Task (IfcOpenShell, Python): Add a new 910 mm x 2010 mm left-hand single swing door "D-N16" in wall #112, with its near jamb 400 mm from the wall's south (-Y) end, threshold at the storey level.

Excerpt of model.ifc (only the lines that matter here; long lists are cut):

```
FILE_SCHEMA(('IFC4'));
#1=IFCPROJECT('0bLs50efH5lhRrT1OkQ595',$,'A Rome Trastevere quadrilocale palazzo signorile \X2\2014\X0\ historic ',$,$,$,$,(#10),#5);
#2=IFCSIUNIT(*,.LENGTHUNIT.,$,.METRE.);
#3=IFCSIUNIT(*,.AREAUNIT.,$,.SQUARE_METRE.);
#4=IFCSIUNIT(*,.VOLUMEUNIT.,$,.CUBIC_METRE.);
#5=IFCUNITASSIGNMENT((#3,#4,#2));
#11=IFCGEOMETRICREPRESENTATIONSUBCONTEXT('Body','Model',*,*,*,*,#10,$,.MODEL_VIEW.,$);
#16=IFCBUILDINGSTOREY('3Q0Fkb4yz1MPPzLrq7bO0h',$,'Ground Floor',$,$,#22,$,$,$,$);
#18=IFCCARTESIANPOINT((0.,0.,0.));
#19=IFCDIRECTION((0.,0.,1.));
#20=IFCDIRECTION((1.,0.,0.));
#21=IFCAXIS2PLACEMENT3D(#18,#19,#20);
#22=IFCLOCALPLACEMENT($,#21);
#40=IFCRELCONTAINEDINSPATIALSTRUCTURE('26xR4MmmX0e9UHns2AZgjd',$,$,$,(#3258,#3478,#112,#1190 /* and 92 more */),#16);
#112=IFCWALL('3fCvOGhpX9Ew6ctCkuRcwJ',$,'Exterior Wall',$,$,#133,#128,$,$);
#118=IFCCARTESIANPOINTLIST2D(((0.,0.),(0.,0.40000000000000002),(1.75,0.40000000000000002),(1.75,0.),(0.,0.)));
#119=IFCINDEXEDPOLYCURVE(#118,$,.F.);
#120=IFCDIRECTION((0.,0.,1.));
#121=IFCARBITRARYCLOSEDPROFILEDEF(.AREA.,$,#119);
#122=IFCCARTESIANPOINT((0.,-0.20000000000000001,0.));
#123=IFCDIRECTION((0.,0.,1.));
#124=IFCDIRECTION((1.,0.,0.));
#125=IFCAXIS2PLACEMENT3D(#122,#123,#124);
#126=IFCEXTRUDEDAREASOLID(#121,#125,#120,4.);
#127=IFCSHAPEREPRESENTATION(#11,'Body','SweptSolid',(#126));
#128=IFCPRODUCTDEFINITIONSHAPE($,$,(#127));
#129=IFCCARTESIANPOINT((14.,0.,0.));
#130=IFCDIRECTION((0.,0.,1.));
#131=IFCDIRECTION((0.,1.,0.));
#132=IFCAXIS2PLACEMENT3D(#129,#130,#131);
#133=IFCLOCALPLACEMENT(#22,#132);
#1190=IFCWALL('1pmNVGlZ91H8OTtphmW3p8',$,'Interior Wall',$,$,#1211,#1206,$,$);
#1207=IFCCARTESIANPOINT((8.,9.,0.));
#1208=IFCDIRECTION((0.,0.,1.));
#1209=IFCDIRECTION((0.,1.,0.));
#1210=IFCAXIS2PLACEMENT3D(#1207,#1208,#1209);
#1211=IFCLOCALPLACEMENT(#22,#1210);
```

```python
import numpy as np
import ifcopenshell
import ifcopenshell.api.feature
import ifcopenshell.api.geometry
import ifcopenshell.api.root
import ifcopenshell.api.spatial
import ifcopenshell.geom
import ifcopenshell.util.element
import ifcopenshell.util.placement
import ifcopenshell.util.representation
import ifcopenshell.util.shape
import ifcopenshell.util.unit

model = ifcopenshell.open("model.ifc")
unit_scale = ifcopenshell.util.unit.calculate_unit_scale(model)
settings = ifcopenshell.geom.settings()


def volume(element):
    """Net volume in cubic metres, openings subtracted."""
    shape = ifcopenshell.geom.create_shape(settings, element)
    return ifcopenshell.util.shape.get_volume(shape.geometry)


wall = model.by_guid("3fCvOGhpX9Ew6ctCkuRcwJ")
storey = ifcopenshell.util.element.get_container(wall, ifc_class="IfcBuildingStorey")
context = ifcopenshell.util.representation.get_context(model, "Model", "Body", "MODEL_VIEW")
before = volume(wall)

width, height, from_end, sill = 0.91, 2.01, 0.4, 0.0  # metres

# The wall runs along its own X axis, and the end named is its -X end.
wall_shape = ifcopenshell.geom.create_shape(settings, wall)
x, y, z = ifcopenshell.util.shape.get_vertices(wall_shape.geometry).T
start = x.min() + from_end
face, thickness = float(y.min()), float(y.max() - y.min())
wall_matrix = ifcopenshell.util.placement.get_local_placement(wall.ObjectPlacement)
level = ifcopenshell.util.placement.get_local_placement(storey.ObjectPlacement)[2, 3]


def in_wall(x, y):
    """Placement at x, y metres in the wall's axes, at sill height."""
    matrix = wall_matrix.copy()
    matrix[:, 3] = wall_matrix @ np.array([x / unit_scale, y / unit_scale, 0.0, 1.0])
    matrix[2, 3] = level + sill / unit_scale
    return matrix


# Opening: a box that overshoots both wall faces by 50 mm.
opening = ifcopenshell.api.root.create_entity(model, ifc_class="IfcOpeningElement", predefined_type="OPENING")
box = ifcopenshell.api.geometry.add_wall_representation(
    model, context=context, length=width, height=height, thickness=thickness + 0.1
)
ifcopenshell.api.geometry.assign_representation(model, product=opening, representation=box)
ifcopenshell.api.geometry.edit_object_placement(model, product=opening, matrix=in_wall(start, face - 0.05), is_si=False)
ifcopenshell.api.feature.add_feature(model, feature=opening, element=wall)

door = ifcopenshell.api.root.create_entity(model, ifc_class="IfcDoor", name="D-N16", predefined_type="DOOR")
door.OverallWidth, door.OverallHeight = width / unit_scale, height / unit_scale
door.OperationType = "SINGLE_SWING_LEFT"
body = ifcopenshell.api.geometry.add_door_representation(
    model,
    context=context,
    overall_width=door.OverallWidth,
    overall_height=door.OverallHeight,
    operation_type="SINGLE_SWING_LEFT",
    lining_properties={"LiningDepth": thickness / unit_scale, "ThresholdDepth": thickness / unit_scale},
)
ifcopenshell.api.geometry.assign_representation(model, product=door, representation=body)
ifcopenshell.api.spatial.assign_container(model, products=[door], relating_structure=storey)
ifcopenshell.api.feature.add_filling(model, opening=opening, element=door)

# The lining spans the wall, so the door starts at the wall face.
ifcopenshell.api.geometry.edit_object_placement(model, product=door, matrix=in_wall(start, face), is_si=False)

after = volume(wall)

print(f"wall volume {before:.3f} -> {after:.3f} m3")

model.write("model_rev.ifc")
```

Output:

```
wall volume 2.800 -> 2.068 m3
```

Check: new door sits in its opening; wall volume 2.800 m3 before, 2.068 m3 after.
